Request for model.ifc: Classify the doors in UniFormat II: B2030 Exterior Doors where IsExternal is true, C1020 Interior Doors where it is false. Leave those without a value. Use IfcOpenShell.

First a look at what the model holds.

```python
import ifcopenshell
import ifcopenshell.util.element

model = ifcopenshell.open("model.ifc")
print(model.schema)
print("classifications:", [c.Name for c in model.by_type("IfcClassification")])
values = [ifcopenshell.util.element.get_pset(e, "Pset_DoorCommon", "IsExternal") for e in model.by_type("IfcDoor")]
for value in (True, False, None):
    print("IsExternal", value, values.count(value))
```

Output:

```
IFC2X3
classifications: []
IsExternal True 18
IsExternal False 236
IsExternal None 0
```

```python
import ifcopenshell
import ifcopenshell.api.classification
import ifcopenshell.util.element

model = ifcopenshell.open("model.ifc")

# IFC2X3 requires Source and Edition and has no link from the project to the system.
system = model.create_entity("IfcClassification", Source="ASTM", Edition="E1557", Name="UniFormat II")

doors = model.by_type("IfcDoor")
external = {e: ifcopenshell.util.element.get_pset(e, "Pset_DoorCommon", "IsExternal") for e in doors}
for flag, code, name in ((True, "B2030", "Exterior Doors"), (False, "C1020", "Interior Doors")):
    products = [e for e in doors if external[e] is flag]
    ifcopenshell.api.classification.add_reference(
        model, products=products, classification=system, identification=code, name=name
    )
    print(code, len(products))

model.write("model_v2.ifc")
```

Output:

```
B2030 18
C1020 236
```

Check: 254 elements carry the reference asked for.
